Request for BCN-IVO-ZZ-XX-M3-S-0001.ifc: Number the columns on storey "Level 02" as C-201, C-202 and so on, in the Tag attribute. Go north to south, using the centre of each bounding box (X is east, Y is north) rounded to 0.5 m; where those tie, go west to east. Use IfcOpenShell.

First a look at what the model holds.

```python
import ifcopenshell
import ifcopenshell.util.element
import ifcopenshell.util.placement

model = ifcopenshell.open("BCN-IVO-ZZ-XX-M3-S-0001.ifc")
print(model.schema)
storey = next(s for s in model.by_type("IfcBuildingStorey") if s.Name == "Level 02")
columns = [e for e in ifcopenshell.util.element.get_decomposition(storey) if e.is_a("IfcColumn")]
for e in sorted(columns, key=lambda e: e.id()):
    origin = ifcopenshell.util.placement.get_local_placement(e.ObjectPlacement)[:3, 3]
    print(e.id(), e.Tag, e.Name, origin.round(2) + 0.0, sep=" | ")
```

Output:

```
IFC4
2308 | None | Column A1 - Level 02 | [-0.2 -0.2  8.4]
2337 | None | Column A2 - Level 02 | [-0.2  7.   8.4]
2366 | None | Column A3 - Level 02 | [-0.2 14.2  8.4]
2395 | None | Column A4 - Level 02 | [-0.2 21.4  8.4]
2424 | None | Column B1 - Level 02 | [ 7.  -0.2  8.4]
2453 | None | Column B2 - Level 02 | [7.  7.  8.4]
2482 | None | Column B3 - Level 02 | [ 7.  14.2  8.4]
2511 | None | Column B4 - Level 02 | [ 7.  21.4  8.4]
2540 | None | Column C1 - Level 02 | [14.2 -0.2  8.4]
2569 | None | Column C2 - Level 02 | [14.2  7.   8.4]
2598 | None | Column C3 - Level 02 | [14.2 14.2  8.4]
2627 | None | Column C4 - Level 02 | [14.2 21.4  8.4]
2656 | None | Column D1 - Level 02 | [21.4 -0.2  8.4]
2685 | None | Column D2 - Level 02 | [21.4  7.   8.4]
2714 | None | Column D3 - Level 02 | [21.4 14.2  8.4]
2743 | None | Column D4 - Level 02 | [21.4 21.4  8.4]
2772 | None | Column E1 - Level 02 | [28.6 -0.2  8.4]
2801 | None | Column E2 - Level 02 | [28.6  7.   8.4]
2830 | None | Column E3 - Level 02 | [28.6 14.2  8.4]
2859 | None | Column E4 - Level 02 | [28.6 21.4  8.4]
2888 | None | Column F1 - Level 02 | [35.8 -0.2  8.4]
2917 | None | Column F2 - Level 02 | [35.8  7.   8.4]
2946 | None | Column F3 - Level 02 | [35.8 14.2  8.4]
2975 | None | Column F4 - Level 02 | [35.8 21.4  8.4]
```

```python
import ifcopenshell
import ifcopenshell.geom
import ifcopenshell.util.element
import ifcopenshell.util.shape

model = ifcopenshell.open("BCN-IVO-ZZ-XX-M3-S-0001.ifc")
settings = ifcopenshell.geom.settings()
settings.set("use-world-coords", True)


def centre(element):
    shape = ifcopenshell.geom.create_shape(settings, element)
    return ifcopenshell.util.shape.get_bbox_centroid(shape.geometry)


storey = next(s for s in model.by_type("IfcBuildingStorey") if s.Name == "Level 02")
columns = [e for e in ifcopenshell.util.element.get_decomposition(storey) if e.is_a("IfcColumn")]

# Insertion points can sit at a corner or the storey origin, so sort by the geometry (in metres).
centres = {e: centre(e) for e in columns}
columns.sort(key=lambda e: (-round(centres[e][1] / 0.5), centres[e][0]))

for i, e in enumerate(columns, start=1):
    number = f"C-2{i:02d}"
    e.Tag = number
    print(e.id(), number)

model.write("BCN-IVO-ZZ-XX-M3-S-0001_v2.ifc")
```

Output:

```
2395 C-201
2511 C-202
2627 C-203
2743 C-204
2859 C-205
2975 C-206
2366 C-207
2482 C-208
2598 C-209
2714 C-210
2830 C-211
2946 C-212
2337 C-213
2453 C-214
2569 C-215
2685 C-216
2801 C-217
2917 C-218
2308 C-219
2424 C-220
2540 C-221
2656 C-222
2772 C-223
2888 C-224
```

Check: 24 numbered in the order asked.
